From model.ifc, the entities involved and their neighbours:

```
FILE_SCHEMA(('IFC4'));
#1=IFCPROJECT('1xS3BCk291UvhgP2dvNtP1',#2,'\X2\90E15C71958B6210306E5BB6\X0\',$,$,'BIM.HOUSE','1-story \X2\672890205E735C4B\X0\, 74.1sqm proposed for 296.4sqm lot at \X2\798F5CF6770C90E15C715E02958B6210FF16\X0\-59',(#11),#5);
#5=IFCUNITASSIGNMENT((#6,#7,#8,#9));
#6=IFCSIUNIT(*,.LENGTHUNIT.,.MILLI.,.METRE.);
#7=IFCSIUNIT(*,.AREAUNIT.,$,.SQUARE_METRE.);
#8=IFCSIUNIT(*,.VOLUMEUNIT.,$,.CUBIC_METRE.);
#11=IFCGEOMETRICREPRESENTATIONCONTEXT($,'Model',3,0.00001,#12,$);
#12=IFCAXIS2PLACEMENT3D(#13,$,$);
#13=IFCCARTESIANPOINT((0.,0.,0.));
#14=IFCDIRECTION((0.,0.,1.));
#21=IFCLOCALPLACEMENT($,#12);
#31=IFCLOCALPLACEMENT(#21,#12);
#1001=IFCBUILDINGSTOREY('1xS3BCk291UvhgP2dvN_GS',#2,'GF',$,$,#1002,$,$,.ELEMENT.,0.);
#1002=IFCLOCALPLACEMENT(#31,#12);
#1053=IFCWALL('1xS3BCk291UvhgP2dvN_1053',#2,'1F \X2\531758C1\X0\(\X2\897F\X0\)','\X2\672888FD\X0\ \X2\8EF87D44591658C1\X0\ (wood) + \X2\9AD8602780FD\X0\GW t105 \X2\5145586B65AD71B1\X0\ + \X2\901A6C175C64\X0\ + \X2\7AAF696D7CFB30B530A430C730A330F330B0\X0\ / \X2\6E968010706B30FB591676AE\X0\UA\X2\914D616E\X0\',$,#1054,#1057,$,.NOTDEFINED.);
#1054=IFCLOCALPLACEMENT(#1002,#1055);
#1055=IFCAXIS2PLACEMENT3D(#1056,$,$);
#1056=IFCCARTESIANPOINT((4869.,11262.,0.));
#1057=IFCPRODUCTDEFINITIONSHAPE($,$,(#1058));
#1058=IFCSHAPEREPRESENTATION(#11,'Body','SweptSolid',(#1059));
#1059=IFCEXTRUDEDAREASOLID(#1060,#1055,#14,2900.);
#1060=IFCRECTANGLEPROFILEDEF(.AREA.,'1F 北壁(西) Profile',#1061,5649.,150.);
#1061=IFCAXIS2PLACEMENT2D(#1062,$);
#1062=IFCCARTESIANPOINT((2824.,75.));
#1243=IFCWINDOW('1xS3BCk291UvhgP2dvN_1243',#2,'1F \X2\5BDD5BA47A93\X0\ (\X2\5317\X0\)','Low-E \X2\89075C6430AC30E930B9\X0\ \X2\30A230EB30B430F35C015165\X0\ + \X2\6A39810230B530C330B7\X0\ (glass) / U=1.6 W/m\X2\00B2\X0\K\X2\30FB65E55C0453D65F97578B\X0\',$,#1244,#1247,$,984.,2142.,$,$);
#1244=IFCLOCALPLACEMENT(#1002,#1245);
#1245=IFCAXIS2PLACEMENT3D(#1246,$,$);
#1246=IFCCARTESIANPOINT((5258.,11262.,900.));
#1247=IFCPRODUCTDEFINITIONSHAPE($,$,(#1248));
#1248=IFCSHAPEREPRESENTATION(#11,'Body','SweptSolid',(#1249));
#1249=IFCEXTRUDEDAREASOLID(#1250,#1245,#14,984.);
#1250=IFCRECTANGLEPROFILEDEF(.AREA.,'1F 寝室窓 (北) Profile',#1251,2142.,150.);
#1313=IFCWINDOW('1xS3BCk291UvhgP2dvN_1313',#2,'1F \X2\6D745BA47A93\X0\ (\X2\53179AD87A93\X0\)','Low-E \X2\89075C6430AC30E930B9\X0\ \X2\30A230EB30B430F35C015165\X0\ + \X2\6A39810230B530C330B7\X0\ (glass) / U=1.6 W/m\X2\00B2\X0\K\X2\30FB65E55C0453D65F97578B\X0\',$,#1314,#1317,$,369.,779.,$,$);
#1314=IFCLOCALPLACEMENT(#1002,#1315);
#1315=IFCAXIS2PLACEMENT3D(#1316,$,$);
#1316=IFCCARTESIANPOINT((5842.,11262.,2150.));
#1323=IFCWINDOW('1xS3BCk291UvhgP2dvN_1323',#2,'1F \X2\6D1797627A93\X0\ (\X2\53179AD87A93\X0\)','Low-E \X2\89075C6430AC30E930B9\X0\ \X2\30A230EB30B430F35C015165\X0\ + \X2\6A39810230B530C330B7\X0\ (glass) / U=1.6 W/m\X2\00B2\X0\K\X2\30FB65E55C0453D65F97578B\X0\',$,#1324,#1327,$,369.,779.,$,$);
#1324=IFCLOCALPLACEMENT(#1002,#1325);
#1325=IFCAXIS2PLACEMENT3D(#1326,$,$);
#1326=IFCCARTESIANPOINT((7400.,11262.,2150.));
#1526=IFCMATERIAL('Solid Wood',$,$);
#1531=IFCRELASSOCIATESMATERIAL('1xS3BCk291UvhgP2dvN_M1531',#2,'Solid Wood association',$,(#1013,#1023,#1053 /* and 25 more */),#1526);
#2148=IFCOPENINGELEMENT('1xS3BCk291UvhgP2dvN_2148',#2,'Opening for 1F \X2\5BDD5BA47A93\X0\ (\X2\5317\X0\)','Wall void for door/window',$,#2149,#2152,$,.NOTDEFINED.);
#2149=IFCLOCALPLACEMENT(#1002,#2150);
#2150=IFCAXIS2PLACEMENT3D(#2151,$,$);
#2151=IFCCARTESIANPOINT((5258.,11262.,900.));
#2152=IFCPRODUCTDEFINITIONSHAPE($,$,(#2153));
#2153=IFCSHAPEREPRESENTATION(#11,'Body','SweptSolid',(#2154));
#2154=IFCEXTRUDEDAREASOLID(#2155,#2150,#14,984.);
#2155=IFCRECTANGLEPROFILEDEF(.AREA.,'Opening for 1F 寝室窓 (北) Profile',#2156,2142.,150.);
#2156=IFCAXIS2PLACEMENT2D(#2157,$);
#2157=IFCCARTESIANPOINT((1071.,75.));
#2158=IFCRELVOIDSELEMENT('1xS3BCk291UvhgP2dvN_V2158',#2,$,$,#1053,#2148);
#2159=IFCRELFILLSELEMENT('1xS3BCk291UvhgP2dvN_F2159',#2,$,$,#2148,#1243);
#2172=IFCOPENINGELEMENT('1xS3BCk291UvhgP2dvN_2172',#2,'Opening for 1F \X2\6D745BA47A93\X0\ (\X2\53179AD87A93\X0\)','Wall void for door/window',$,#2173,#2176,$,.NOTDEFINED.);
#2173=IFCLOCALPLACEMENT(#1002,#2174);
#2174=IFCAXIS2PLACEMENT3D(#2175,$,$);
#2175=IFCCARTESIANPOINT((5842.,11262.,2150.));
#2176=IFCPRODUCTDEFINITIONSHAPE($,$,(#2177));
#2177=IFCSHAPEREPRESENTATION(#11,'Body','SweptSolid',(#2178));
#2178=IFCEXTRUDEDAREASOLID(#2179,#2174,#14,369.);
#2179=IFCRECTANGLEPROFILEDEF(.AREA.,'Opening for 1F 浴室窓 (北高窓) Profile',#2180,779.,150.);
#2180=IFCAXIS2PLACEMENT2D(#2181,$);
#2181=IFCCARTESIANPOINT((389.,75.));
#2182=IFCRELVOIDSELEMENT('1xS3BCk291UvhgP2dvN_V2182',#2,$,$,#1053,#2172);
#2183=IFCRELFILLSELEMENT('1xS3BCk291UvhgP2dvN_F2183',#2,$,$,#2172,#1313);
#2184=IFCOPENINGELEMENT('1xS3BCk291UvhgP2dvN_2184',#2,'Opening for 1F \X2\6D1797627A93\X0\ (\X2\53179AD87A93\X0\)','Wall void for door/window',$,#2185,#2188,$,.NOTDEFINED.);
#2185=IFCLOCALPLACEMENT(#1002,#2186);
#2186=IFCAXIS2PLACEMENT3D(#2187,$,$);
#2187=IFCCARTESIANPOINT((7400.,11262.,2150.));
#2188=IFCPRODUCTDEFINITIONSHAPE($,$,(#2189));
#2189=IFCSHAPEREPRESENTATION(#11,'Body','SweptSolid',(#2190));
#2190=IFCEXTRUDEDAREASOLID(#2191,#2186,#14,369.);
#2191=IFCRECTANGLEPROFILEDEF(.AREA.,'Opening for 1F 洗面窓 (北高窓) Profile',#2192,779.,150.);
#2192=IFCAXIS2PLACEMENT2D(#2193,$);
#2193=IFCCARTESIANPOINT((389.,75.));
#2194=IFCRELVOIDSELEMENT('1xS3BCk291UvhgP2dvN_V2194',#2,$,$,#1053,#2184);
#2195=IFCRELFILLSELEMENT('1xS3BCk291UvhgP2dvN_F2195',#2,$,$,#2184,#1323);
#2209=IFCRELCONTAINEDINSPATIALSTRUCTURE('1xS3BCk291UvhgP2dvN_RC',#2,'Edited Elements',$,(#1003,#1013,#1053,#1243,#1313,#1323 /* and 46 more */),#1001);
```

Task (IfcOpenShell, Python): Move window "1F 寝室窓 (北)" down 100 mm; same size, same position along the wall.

```python
import numpy as np
import ifcopenshell
import ifcopenshell.api.geometry
import ifcopenshell.util.placement
import ifcopenshell.util.unit

model = ifcopenshell.open("model.ifc")
unit_scale = ifcopenshell.util.unit.calculate_unit_scale(model)

window = model.by_guid("1xS3BCk291UvhgP2dvN_1243")
opening = window.FillsVoids[0].RelatingOpeningElement
dz = -100.0

shift = np.array([0.0, 0.0, dz])
# The window is not placed relative to its opening, so move both.
for product in (opening, window):
    matrix = ifcopenshell.util.placement.get_local_placement(product.ObjectPlacement)
    matrix[:3, 3] += shift
    ifcopenshell.api.geometry.edit_object_placement(model, product=product, matrix=matrix, is_si=False)

print(f"moved by {dz * unit_scale:+.3f} m")

model.write("model_v2.ifc")
```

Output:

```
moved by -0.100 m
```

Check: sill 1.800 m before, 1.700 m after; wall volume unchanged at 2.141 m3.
